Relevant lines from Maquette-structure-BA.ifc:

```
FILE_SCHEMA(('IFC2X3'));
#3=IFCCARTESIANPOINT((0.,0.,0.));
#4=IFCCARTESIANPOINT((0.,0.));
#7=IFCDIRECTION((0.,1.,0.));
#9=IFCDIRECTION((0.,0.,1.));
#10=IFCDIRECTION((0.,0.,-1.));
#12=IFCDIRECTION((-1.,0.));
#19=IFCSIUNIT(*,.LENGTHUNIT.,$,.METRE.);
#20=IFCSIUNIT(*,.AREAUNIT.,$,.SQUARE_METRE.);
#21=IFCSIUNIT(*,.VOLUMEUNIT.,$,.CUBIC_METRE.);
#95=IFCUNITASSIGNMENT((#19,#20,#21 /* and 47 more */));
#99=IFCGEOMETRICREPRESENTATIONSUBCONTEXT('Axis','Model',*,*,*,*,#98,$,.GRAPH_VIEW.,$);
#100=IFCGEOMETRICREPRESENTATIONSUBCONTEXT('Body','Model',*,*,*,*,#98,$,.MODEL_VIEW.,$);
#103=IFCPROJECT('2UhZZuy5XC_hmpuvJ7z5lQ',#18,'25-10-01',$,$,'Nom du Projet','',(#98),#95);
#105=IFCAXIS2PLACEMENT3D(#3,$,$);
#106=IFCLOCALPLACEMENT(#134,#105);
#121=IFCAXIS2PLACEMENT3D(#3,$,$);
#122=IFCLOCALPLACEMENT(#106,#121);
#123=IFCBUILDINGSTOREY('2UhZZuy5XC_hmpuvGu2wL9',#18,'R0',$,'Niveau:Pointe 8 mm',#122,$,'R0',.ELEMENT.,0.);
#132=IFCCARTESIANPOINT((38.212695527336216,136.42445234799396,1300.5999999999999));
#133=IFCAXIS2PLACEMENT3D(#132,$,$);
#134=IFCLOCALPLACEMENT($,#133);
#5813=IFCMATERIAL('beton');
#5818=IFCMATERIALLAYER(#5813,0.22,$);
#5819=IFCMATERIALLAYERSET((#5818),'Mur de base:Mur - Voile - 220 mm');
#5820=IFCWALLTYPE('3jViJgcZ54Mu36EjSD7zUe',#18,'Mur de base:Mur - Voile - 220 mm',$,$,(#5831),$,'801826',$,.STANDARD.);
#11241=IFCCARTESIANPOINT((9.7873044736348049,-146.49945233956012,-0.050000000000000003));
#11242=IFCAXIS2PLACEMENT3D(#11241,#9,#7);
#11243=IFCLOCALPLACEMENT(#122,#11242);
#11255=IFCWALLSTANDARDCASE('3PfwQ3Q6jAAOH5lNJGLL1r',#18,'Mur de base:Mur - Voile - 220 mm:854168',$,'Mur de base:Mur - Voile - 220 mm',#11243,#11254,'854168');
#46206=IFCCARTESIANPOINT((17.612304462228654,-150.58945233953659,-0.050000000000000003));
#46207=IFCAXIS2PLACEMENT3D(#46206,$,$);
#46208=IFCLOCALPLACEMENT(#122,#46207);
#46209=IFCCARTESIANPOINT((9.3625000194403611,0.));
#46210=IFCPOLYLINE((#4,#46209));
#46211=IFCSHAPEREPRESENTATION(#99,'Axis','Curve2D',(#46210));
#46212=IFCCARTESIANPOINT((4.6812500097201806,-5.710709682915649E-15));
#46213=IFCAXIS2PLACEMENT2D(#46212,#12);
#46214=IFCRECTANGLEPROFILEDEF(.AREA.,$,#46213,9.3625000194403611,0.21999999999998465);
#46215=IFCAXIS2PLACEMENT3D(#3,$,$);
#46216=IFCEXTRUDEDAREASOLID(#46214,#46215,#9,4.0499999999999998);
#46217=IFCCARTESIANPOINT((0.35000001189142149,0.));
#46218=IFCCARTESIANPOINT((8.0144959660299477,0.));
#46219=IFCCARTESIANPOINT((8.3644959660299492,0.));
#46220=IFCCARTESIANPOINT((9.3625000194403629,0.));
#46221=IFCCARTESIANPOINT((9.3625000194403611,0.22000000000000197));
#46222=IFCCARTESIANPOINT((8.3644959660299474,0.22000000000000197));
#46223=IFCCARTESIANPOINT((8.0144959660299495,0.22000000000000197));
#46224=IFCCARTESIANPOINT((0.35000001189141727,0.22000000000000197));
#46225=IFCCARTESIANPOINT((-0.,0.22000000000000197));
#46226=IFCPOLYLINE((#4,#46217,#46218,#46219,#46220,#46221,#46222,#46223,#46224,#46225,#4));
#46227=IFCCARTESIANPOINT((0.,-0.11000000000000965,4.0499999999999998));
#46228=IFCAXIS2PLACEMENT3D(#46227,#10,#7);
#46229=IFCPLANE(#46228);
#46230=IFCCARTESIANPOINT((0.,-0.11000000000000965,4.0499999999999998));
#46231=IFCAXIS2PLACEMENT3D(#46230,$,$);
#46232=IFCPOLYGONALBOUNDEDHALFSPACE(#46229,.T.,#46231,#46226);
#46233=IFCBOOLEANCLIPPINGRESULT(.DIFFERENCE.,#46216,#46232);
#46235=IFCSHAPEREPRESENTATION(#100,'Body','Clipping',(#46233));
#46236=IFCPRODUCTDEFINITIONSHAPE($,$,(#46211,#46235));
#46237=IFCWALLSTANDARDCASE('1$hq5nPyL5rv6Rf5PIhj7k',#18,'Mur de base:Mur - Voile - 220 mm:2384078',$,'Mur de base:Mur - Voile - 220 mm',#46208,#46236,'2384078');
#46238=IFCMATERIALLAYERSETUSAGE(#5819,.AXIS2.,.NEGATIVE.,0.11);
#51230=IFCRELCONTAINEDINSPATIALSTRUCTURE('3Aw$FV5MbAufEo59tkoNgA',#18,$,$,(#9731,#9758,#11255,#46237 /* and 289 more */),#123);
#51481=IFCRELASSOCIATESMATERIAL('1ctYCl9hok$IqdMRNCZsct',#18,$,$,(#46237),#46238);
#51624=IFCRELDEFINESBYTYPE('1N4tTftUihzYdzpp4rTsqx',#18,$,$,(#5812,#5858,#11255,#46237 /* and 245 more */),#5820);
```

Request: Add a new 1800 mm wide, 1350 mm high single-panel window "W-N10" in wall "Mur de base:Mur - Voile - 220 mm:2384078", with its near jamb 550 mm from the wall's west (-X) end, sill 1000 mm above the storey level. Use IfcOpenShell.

```python
import numpy as np
import ifcopenshell
import ifcopenshell.api.feature
import ifcopenshell.api.geometry
import ifcopenshell.api.root
import ifcopenshell.api.spatial
import ifcopenshell.api.type
import ifcopenshell.geom
import ifcopenshell.util.element
import ifcopenshell.util.placement
import ifcopenshell.util.representation
import ifcopenshell.util.shape
import ifcopenshell.util.unit

model = ifcopenshell.open("Maquette-structure-BA.ifc")
unit_scale = ifcopenshell.util.unit.calculate_unit_scale(model)
settings = ifcopenshell.geom.settings()


def volume(element):
    """Net volume in cubic metres, openings subtracted."""
    shape = ifcopenshell.geom.create_shape(settings, element)
    return ifcopenshell.util.shape.get_volume(shape.geometry)


wall = model.by_guid("1$hq5nPyL5rv6Rf5PIhj7k")
storey = ifcopenshell.util.element.get_container(wall, ifc_class="IfcBuildingStorey")
context = ifcopenshell.util.representation.get_context(model, "Model", "Body", "MODEL_VIEW")
before = volume(wall)

width, height, from_end, sill = 1.8, 1.35, 0.55, 1  # metres

# The wall runs along its own X axis, and the end named is its -X end.
wall_shape = ifcopenshell.geom.create_shape(settings, wall)
x, y, z = ifcopenshell.util.shape.get_vertices(wall_shape.geometry).T
start = x.min() + from_end
face, thickness = float(y.min()), float(y.max() - y.min())
wall_matrix = ifcopenshell.util.placement.get_local_placement(wall.ObjectPlacement)
level = ifcopenshell.util.placement.get_local_placement(storey.ObjectPlacement)[2, 3]


def in_wall(x, y):
    """Placement at x, y metres in the wall's axes, at sill height."""
    matrix = wall_matrix.copy()
    matrix[:, 3] = wall_matrix @ np.array([x / unit_scale, y / unit_scale, 0.0, 1.0])
    matrix[2, 3] = level + sill / unit_scale
    return matrix


# Opening: a box that overshoots both wall faces by 50 mm.
opening = ifcopenshell.api.root.create_entity(model, ifc_class="IfcOpeningElement")
box = ifcopenshell.api.geometry.add_wall_representation(
    model, context=context, length=width, height=height, thickness=thickness + 0.1
)
ifcopenshell.api.geometry.assign_representation(model, product=opening, representation=box)
ifcopenshell.api.geometry.edit_object_placement(model, product=opening, matrix=in_wall(start, face - 0.05), is_si=False)
ifcopenshell.api.feature.add_feature(model, feature=opening, element=wall)

window = ifcopenshell.api.root.create_entity(model, ifc_class="IfcWindow", name="W-N10")
window.OverallWidth, window.OverallHeight = width / unit_scale, height / unit_scale
body = ifcopenshell.api.geometry.add_window_representation(
    model,
    context=context,
    overall_width=window.OverallWidth,
    overall_height=window.OverallHeight,
    partition_type="SINGLE_PANEL",
)
ifcopenshell.api.geometry.assign_representation(model, product=window, representation=body)
ifcopenshell.api.spatial.assign_container(model, products=[window], relating_structure=storey)
fills = ifcopenshell.api.feature.add_filling(model, opening=opening, element=window)
fills.OwnerHistory = window.OwnerHistory  # required in IFC2X3

# IFC2X3 keeps the operation on the window style.
style = ifcopenshell.api.root.create_entity(model, ifc_class="IfcWindowStyle", name="W-N10")
style.OperationType, style.ConstructionType = "SINGLE_PANEL", "NOTDEFINED"
style.ParameterTakesPrecedence = style.Sizeable = False
ifcopenshell.api.type.assign_type(model, related_objects=[window], relating_type=style)

# Centre the window in the wall's thickness.
ifcopenshell.api.geometry.edit_object_placement(model, product=window, matrix=in_wall(start, face), is_si=False)
window_shape = ifcopenshell.geom.create_shape(settings, window)
depth = ifcopenshell.util.shape.get_vertices(window_shape.geometry)[:, 1]
offset = face + thickness / 2 - (depth.min() + depth.max()) / 2
ifcopenshell.api.geometry.edit_object_placement(model, product=window, matrix=in_wall(start, offset), is_si=False)

after = volume(wall)

print(f"wall volume {before:.3f} -> {after:.3f} m3")

model.write("Maquette-structure-BA-out.ifc")
```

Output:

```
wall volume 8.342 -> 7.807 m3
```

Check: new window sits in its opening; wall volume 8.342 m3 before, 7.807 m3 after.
